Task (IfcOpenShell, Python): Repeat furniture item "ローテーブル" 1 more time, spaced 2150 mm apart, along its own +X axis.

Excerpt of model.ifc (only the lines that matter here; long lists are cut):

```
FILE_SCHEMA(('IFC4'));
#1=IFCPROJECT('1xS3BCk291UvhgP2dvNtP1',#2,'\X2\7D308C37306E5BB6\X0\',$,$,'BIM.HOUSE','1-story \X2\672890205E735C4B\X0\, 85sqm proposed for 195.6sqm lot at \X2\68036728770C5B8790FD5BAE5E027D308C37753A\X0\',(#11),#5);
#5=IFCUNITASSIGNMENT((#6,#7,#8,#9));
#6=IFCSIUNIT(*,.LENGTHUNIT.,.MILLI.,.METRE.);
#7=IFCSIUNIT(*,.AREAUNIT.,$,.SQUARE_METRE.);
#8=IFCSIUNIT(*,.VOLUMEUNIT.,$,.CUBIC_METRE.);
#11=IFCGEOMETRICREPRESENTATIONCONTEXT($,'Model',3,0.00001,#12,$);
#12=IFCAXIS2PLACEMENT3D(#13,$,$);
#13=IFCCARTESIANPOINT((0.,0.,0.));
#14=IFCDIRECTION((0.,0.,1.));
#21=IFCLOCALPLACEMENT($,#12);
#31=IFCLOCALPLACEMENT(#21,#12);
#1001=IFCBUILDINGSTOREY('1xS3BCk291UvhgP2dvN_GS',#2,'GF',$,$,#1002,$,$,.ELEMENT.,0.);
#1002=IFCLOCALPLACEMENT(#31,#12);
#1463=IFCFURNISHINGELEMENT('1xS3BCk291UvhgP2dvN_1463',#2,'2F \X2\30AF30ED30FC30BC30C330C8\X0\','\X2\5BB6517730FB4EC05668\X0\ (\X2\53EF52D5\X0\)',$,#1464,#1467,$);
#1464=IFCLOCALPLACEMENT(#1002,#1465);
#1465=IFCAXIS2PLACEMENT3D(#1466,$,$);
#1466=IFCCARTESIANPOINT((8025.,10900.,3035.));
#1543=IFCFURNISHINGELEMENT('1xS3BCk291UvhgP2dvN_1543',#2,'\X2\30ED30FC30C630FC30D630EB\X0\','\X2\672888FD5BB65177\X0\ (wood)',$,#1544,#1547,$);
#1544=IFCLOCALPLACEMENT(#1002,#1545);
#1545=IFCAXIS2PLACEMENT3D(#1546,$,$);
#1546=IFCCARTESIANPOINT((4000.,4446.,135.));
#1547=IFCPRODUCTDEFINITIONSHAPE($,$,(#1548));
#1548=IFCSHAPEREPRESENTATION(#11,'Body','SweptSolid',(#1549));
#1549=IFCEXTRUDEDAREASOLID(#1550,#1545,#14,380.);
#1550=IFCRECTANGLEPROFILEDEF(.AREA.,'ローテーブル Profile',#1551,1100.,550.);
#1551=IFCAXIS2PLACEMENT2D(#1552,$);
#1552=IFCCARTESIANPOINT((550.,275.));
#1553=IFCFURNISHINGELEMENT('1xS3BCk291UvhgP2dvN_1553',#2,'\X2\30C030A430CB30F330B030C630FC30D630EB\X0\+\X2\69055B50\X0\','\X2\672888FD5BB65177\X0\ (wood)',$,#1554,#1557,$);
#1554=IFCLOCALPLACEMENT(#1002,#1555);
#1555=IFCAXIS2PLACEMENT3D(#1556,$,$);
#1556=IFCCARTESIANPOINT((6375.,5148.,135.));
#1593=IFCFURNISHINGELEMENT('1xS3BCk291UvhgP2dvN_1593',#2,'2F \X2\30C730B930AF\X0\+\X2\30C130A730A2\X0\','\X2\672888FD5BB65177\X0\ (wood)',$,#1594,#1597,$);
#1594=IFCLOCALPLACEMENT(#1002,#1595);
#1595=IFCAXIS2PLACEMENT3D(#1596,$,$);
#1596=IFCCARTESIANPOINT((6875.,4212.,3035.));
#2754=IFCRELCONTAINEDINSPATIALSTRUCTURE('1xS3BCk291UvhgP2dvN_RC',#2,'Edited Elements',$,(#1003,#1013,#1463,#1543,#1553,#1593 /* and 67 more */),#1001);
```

```python
import ifcopenshell
import ifcopenshell.api.geometry
import ifcopenshell.api.root
import ifcopenshell.util.element
import ifcopenshell.util.placement

model = ifcopenshell.open("model.ifc")


def reuse_history(source, copy):
    """copy_class also copies each property set's owner history, people and application; keep the originals."""
    for rel in copy.IsDefinedBy:
        if rel.is_a("IfcRelDefinesByProperties") and (history := rel.RelatingPropertyDefinition.OwnerHistory):
            rel.RelatingPropertyDefinition.OwnerHistory = source.OwnerHistory
            ifcopenshell.util.element.remove_deep2(model, history)


source = model.by_guid("1xS3BCk291UvhgP2dvN_1543")
base = ifcopenshell.util.placement.get_local_placement(source.ObjectPlacement)
step = base[:3, 0] * 2150.0

for i in range(1, 2):
    copy = ifcopenshell.api.root.copy_class(model, product=source)
    copy.Representation = ifcopenshell.util.element.copy_deep(
        model, source.Representation, exclude=["IfcGeometricRepresentationContext", "IfcRepresentationMap"]
    )
    reuse_history(source, copy)
    matrix = base.copy()
    matrix[:3, 3] += i * step
    print("added at", matrix[:3, 3].round(3) + 0.0)
    ifcopenshell.api.geometry.edit_object_placement(model, product=copy, matrix=matrix, is_si=False)

model.write("model_v2.ifc")
```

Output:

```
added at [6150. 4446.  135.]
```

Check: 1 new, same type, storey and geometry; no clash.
